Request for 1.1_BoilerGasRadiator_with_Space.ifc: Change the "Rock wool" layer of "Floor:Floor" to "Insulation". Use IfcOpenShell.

First a look at what the model holds.

```python
import ifcopenshell
import ifcopenshell.util.element

model = ifcopenshell.open("1.1_BoilerGasRadiator_with_Space.ifc")
print(model.schema)
for layer_set in model.by_type("IfcMaterialLayerSet"):
    if layer_set.LayerSetName == "Floor:Floor":
        for layer in layer_set.MaterialLayers:
            print(layer.id(), layer.Material and layer.Material.Name, layer.LayerThickness, sep=" | ")
        print(len(ifcopenshell.util.element.get_elements_by_material(model, layer_set)), "elements and types use it")
print(sorted(m.Name for m in model.by_type("IfcMaterial") if m.Name)[:60])
```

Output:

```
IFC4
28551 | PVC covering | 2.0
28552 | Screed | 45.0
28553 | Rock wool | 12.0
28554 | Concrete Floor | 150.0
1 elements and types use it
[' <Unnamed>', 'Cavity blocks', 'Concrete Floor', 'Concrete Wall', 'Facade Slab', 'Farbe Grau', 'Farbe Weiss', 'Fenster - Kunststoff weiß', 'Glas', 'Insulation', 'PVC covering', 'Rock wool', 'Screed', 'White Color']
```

```python
import ifcopenshell
import ifcopenshell.api.material

model = ifcopenshell.open("1.1_BoilerGasRadiator_with_Space.ifc")

layer_set = next(s for s in model.by_type("IfcMaterialLayerSet") if s.LayerSetName == "Floor:Floor")
layer = next(l for l in layer_set.MaterialLayers if l.Material and l.Material.Name == "Rock wool")
material = next(m for m in model.by_type("IfcMaterial") if m.Name == "Insulation")

# Point this one layer at the other material; renaming the old one would change it everywhere.
ifcopenshell.api.material.edit_layer(model, layer=layer, attributes={}, material=material)

print([l.Material.Name if l.Material else None for l in layer_set.MaterialLayers])

model.write("1.1_BoilerGasRadiator_with_Space_v2.ifc")
```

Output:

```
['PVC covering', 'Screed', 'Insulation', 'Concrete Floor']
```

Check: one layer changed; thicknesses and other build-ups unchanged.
